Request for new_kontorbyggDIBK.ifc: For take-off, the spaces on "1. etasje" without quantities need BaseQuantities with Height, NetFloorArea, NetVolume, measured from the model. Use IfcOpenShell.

First a look at what the model holds.

```python
import ifcopenshell
import ifcopenshell.util.element
import ifcopenshell.util.unit

model = ifcopenshell.open("new_kontorbyggDIBK.ifc")
print(model.schema)
for unit_type in ("LENGTHUNIT", "AREAUNIT", "VOLUMEUNIT"):
    print(unit_type, ifcopenshell.util.unit.calculate_unit_scale(model, unit_type))
storey = next(s for s in model.by_type("IfcBuildingStorey") if s.Name == "1. etasje")
spaces = [e for e in ifcopenshell.util.element.get_decomposition(storey) if e.is_a("IfcSpace")]
for e in sorted(spaces, key=lambda e: e.id()):
    print(e.id(), e.is_a(), e.Name, list(ifcopenshell.util.element.get_psets(e, qtos_only=True)), sep=" | ")
```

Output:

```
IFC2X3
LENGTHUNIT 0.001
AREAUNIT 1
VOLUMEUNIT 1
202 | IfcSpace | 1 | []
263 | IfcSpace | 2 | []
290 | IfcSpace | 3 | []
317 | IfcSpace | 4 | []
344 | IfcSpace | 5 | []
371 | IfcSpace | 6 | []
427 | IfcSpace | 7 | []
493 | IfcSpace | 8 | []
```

```python
import ifcopenshell
import ifcopenshell.api.pset
import ifcopenshell.geom
import ifcopenshell.util.element
import ifcopenshell.util.shape
import ifcopenshell.util.unit

model = ifcopenshell.open("new_kontorbyggDIBK.ifc")
unit_scale = ifcopenshell.util.unit.calculate_unit_scale(model)
area_scale = ifcopenshell.util.unit.calculate_unit_scale(model, "AREAUNIT")
volume_scale = ifcopenshell.util.unit.calculate_unit_scale(model, "VOLUMEUNIT")
settings = ifcopenshell.geom.settings()

storey = next(s for s in model.by_type("IfcBuildingStorey") if s.Name == "1. etasje")
spaces = [e for e in ifcopenshell.util.element.get_decomposition(storey) if e.is_a("IfcSpace")]

for e in sorted(spaces, key=lambda e: e.id()):
    if ifcopenshell.util.element.get_psets(e, qtos_only=True, should_inherit=False):
        continue
    # Geometry comes back in metres, in the element's own axes.
    shape = ifcopenshell.geom.create_shape(settings, e)
    values = {
        "Height": ifcopenshell.util.shape.get_z(shape.geometry) / unit_scale,
        "NetFloorArea": ifcopenshell.util.shape.get_footprint_area(shape.geometry) / area_scale,
        "NetVolume": ifcopenshell.util.shape.get_volume(shape.geometry) / volume_scale,
    }
    qto = ifcopenshell.api.pset.add_qto(model, product=e, name="BaseQuantities")
    ifcopenshell.api.pset.edit_qto(model, qto=qto, properties=values)
    print(e.id(), {k: round(v, 3) for k, v in values.items()})

model.write("new_kontorbyggDIBK_rev.ifc")
```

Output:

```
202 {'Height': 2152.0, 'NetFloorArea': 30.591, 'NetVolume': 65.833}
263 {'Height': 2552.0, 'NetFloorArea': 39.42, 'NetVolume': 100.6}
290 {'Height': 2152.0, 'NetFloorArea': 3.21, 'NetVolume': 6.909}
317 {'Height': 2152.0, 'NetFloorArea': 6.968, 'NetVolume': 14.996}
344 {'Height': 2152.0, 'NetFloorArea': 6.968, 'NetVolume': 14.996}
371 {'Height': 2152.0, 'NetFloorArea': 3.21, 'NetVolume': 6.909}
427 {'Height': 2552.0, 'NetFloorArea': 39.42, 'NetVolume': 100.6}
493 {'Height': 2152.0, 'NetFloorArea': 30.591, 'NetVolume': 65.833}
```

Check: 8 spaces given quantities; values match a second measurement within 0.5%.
